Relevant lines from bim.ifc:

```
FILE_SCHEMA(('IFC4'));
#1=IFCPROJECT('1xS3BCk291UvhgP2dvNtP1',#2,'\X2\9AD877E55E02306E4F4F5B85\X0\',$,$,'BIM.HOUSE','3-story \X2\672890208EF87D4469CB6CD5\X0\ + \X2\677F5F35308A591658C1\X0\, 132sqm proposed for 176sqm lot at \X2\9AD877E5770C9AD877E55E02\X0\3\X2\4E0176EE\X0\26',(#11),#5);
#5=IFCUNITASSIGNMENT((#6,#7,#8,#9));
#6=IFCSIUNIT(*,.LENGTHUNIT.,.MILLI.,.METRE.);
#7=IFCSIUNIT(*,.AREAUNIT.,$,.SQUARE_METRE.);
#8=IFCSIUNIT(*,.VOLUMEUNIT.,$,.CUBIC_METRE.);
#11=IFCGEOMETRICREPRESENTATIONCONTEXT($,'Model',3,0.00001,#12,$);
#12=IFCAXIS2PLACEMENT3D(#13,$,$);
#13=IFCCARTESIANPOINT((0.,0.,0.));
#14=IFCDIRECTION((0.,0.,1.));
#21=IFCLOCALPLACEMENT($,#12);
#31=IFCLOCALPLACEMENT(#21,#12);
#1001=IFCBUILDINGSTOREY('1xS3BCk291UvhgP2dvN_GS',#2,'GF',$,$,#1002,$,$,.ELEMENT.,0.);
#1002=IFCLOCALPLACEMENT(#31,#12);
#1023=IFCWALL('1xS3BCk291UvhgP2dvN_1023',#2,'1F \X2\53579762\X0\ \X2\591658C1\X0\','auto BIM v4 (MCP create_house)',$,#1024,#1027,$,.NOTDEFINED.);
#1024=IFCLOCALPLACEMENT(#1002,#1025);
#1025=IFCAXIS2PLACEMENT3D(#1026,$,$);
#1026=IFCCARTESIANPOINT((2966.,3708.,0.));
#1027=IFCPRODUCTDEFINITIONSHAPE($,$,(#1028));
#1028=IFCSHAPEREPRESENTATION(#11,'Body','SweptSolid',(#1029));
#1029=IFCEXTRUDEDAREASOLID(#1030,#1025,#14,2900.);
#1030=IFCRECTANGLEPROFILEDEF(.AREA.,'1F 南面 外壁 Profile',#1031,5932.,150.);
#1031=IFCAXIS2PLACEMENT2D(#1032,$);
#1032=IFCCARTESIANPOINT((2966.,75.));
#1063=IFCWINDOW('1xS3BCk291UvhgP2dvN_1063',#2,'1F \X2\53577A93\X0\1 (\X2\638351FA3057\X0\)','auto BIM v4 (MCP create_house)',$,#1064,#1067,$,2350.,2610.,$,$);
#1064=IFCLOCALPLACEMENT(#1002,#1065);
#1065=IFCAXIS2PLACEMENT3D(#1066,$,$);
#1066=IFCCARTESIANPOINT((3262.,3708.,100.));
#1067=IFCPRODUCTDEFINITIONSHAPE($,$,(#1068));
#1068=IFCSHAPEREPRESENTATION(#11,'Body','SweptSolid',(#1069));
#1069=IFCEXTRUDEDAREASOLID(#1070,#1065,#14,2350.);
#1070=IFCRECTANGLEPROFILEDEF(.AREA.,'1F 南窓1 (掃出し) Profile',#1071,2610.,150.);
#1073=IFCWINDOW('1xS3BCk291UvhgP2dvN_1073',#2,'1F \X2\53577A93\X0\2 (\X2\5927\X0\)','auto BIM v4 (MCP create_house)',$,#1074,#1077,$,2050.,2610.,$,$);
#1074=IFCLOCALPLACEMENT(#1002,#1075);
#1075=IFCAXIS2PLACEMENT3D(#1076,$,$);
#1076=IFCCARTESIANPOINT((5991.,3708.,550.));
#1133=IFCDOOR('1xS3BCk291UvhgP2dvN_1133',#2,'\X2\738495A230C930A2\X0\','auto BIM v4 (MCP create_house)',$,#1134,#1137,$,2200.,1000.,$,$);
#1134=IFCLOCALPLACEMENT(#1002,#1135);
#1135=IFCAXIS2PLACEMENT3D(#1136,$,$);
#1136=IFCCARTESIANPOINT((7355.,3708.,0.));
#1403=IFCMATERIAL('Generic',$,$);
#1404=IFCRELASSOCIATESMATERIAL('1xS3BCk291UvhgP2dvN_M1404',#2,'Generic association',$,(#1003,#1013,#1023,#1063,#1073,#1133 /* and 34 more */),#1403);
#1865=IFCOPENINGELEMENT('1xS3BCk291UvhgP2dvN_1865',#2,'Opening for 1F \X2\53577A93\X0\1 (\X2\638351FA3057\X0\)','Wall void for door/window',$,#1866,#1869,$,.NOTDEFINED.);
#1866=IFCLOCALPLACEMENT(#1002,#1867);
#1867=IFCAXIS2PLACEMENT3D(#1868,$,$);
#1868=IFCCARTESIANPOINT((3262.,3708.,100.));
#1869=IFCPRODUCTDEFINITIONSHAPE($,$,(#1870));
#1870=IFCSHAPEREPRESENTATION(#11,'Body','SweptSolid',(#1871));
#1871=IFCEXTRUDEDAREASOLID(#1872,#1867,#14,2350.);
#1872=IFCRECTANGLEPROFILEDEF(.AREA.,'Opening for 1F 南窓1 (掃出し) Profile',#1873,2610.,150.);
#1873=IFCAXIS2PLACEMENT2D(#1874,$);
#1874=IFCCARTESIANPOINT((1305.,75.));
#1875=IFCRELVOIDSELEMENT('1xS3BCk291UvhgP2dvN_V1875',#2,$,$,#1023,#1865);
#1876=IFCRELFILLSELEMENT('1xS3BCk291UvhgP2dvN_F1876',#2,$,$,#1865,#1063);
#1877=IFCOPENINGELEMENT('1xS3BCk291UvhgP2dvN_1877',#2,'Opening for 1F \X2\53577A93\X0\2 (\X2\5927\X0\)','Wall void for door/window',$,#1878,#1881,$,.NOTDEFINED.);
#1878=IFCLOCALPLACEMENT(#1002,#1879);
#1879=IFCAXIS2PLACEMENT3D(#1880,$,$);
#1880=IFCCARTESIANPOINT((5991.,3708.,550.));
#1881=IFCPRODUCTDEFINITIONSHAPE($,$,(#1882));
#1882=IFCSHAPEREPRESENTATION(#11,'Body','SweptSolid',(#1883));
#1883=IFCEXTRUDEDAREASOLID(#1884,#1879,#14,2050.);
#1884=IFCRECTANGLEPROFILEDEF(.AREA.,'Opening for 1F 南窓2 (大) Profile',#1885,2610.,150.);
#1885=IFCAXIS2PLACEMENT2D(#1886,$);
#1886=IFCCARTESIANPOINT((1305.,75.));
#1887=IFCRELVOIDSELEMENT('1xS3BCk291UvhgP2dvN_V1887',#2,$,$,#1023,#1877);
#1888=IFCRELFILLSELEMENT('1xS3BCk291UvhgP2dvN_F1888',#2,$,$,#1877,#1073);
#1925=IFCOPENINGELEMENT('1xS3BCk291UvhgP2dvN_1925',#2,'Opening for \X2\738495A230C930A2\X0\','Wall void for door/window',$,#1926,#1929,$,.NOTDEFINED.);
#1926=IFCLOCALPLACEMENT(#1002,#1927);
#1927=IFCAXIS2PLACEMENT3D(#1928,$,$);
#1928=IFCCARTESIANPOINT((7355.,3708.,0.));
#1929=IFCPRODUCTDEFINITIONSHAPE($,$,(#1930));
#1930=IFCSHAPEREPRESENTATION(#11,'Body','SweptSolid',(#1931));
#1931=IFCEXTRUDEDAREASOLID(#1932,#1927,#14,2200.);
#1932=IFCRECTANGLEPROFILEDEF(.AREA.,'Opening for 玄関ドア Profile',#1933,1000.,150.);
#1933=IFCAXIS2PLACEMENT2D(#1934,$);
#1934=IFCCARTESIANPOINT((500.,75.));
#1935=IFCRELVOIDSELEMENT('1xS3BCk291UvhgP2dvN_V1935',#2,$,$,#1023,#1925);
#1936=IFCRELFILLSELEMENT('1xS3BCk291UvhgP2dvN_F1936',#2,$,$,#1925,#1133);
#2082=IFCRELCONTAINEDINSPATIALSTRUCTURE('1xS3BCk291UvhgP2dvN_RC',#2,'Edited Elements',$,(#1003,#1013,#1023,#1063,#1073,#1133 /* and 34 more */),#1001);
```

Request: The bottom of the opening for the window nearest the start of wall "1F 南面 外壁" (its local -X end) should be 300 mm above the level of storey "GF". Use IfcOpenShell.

```python
import numpy as np
import ifcopenshell
import ifcopenshell.api.geometry
import ifcopenshell.geom
import ifcopenshell.util.element
import ifcopenshell.util.placement
import ifcopenshell.util.shape
import ifcopenshell.util.unit

model = ifcopenshell.open("bim.ifc")
unit_scale = ifcopenshell.util.unit.calculate_unit_scale(model)

window = model.by_guid("1xS3BCk291UvhgP2dvN_1063")
opening = window.FillsVoids[0].RelatingOpeningElement
storey = ifcopenshell.util.element.get_container(window, ifc_class="IfcBuildingStorey")
level = ifcopenshell.util.placement.get_local_placement(storey.ObjectPlacement)[2, 3]

# The opening's origin need not be at the sill, so measure its lowest point.
shape = ifcopenshell.geom.create_shape(ifcopenshell.geom.settings(), opening)
bottom = ifcopenshell.util.shape.get_shape_bottom_elevation(shape, shape.geometry) / unit_scale
dz = level + 300.0 - bottom

shift = np.array([0.0, 0.0, dz])
# The window is not placed relative to its opening, so move both.
for product in (opening, window):
    matrix = ifcopenshell.util.placement.get_local_placement(product.ObjectPlacement)
    matrix[:3, 3] += shift
    ifcopenshell.api.geometry.edit_object_placement(model, product=product, matrix=matrix, is_si=False)

print(f"moved by {dz * unit_scale:+.3f} m")

model.write("bim-out.ifc")
```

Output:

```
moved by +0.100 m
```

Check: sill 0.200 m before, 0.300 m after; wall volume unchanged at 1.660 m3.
